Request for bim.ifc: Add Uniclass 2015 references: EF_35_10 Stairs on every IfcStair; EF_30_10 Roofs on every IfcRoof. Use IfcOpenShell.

First a look at what the model holds.

```python
import ifcopenshell

model = ifcopenshell.open("bim.ifc")
print(model.schema)
print("classifications:", [c.Name for c in model.by_type("IfcClassification")])
for ifc_class in ("IfcDoor", "IfcRoof", "IfcStair", "IfcWall", "IfcWindow"):
    print(ifc_class, len(model.by_type(ifc_class)))
```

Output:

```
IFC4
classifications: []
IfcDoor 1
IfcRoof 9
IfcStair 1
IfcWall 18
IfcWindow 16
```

```python
import ifcopenshell
import ifcopenshell.api.classification

model = ifcopenshell.open("bim.ifc")

system = ifcopenshell.api.classification.add_classification(model, classification="Uniclass 2015")

codes = {
    "IfcStair": ("EF_35_10", "Stairs"),
    "IfcRoof": ("EF_30_10", "Roofs"),
}
for ifc_class, (code, name) in codes.items():
    products = model.by_type(ifc_class)
    ifcopenshell.api.classification.add_reference(
        model, products=products, classification=system, identification=code, name=name
    )
    print(code, len(products))

model.write("bim_edited.ifc")
```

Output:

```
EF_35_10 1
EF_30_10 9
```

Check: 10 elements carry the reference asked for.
